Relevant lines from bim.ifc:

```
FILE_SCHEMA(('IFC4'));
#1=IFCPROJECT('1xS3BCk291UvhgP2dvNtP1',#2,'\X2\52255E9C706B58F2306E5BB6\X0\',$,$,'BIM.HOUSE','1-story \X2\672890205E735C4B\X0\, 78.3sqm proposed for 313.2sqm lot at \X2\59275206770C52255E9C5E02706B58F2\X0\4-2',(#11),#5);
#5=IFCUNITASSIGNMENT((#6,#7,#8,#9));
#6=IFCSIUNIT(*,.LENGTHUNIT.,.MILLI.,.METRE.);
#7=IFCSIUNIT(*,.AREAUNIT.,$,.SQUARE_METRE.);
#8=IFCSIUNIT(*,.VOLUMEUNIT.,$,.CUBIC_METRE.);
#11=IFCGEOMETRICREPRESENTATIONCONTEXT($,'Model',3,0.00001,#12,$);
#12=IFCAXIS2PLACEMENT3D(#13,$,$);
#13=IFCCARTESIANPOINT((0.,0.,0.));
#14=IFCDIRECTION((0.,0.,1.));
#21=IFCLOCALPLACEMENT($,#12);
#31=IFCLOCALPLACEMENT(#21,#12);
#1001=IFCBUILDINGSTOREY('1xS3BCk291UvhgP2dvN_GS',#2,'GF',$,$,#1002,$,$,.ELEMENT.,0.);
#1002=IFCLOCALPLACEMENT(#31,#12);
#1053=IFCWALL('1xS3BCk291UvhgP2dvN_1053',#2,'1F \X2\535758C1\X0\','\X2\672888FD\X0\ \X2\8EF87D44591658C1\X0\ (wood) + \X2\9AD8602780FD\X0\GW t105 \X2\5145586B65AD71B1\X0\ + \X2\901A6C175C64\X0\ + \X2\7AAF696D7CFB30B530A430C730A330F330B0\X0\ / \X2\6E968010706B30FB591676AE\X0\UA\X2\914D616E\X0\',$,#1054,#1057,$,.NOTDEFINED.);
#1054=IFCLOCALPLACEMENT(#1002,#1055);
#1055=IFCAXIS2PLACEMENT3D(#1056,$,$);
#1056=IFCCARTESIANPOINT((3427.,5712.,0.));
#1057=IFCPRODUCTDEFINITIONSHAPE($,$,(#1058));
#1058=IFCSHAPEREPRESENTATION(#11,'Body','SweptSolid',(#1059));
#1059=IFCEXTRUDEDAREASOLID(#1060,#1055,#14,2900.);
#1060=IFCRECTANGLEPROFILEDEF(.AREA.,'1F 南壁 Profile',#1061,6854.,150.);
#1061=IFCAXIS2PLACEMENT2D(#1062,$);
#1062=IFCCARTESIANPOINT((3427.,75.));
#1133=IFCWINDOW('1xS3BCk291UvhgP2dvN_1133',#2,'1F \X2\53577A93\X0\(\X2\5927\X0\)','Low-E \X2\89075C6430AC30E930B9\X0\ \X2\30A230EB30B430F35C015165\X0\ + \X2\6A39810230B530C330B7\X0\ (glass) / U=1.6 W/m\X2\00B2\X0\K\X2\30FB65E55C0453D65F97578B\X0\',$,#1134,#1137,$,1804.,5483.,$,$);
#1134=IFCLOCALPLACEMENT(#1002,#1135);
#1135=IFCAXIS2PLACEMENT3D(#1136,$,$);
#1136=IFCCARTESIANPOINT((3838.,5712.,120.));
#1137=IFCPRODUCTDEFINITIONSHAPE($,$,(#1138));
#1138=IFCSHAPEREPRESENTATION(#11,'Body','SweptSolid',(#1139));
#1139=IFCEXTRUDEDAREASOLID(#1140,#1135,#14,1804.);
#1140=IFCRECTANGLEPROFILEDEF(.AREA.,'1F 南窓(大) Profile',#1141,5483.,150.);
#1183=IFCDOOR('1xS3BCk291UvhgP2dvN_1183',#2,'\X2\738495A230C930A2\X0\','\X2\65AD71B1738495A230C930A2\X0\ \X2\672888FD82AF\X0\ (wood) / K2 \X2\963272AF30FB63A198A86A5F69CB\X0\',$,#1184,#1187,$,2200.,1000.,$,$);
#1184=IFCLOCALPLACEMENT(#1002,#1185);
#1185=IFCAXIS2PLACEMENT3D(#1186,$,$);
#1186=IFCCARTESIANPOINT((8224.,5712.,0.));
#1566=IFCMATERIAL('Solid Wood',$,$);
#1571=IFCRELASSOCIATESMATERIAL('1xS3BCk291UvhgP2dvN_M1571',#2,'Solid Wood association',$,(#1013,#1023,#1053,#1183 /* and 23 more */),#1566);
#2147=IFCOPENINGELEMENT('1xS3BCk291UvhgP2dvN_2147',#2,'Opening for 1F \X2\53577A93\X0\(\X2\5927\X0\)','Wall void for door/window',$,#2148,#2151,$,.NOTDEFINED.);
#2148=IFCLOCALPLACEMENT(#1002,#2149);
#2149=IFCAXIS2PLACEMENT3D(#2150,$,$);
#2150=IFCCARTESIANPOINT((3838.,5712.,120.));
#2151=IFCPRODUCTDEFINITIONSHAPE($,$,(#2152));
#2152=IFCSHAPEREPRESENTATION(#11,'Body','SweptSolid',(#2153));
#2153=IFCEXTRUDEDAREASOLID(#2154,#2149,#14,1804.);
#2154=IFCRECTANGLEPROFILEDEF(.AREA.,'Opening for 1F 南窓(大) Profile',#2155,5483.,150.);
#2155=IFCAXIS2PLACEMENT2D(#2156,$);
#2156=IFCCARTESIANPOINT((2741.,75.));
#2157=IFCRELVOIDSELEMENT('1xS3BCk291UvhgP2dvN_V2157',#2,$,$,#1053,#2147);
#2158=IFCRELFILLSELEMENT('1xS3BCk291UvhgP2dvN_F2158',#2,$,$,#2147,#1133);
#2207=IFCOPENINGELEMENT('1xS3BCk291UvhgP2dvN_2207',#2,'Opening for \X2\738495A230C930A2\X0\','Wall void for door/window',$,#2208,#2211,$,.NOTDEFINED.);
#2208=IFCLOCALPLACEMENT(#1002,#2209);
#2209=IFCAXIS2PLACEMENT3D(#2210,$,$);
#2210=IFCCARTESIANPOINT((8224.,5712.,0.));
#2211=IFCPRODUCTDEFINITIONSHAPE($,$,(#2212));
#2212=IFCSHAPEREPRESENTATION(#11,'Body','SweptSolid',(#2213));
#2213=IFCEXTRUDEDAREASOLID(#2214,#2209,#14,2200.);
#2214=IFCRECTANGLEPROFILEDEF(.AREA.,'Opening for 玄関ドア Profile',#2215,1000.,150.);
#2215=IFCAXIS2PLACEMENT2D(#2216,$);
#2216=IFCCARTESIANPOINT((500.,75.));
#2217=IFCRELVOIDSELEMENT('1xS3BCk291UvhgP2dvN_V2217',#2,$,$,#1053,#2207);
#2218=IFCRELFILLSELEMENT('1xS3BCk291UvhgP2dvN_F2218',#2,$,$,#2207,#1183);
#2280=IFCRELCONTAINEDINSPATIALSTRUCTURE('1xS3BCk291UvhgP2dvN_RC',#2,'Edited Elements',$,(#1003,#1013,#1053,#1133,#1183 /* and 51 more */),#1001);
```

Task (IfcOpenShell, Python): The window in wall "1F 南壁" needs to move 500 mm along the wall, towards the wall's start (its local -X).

```python
import ifcopenshell
import ifcopenshell.api.geometry
import ifcopenshell.util.placement
import ifcopenshell.util.unit

model = ifcopenshell.open("bim.ifc")
unit_scale = ifcopenshell.util.unit.calculate_unit_scale(model)

window = model.by_guid("1xS3BCk291UvhgP2dvN_1133")
opening = window.FillsVoids[0].RelatingOpeningElement
wall = opening.VoidsElements[0].RelatingBuildingElement

wall_matrix = ifcopenshell.util.placement.get_local_placement(wall.ObjectPlacement)
shift = wall_matrix[:3, 0] * -0.5 / unit_scale
before = ifcopenshell.util.placement.get_local_placement(window.ObjectPlacement)[:3, 3].copy()

# The window is not placed relative to its opening, so move both.
for product in (opening, window):
    matrix = ifcopenshell.util.placement.get_local_placement(product.ObjectPlacement)
    matrix[:3, 3] += shift
    ifcopenshell.api.geometry.edit_object_placement(model, product=product, matrix=matrix, is_si=False)

after = ifcopenshell.util.placement.get_local_placement(window.ObjectPlacement)[:3, 3]
print("window moved by", (after - before).round(3) + 0.0)

model.write("bim_v2.ifc")
```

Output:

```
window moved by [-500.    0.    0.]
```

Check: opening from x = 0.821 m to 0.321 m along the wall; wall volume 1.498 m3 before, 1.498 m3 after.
